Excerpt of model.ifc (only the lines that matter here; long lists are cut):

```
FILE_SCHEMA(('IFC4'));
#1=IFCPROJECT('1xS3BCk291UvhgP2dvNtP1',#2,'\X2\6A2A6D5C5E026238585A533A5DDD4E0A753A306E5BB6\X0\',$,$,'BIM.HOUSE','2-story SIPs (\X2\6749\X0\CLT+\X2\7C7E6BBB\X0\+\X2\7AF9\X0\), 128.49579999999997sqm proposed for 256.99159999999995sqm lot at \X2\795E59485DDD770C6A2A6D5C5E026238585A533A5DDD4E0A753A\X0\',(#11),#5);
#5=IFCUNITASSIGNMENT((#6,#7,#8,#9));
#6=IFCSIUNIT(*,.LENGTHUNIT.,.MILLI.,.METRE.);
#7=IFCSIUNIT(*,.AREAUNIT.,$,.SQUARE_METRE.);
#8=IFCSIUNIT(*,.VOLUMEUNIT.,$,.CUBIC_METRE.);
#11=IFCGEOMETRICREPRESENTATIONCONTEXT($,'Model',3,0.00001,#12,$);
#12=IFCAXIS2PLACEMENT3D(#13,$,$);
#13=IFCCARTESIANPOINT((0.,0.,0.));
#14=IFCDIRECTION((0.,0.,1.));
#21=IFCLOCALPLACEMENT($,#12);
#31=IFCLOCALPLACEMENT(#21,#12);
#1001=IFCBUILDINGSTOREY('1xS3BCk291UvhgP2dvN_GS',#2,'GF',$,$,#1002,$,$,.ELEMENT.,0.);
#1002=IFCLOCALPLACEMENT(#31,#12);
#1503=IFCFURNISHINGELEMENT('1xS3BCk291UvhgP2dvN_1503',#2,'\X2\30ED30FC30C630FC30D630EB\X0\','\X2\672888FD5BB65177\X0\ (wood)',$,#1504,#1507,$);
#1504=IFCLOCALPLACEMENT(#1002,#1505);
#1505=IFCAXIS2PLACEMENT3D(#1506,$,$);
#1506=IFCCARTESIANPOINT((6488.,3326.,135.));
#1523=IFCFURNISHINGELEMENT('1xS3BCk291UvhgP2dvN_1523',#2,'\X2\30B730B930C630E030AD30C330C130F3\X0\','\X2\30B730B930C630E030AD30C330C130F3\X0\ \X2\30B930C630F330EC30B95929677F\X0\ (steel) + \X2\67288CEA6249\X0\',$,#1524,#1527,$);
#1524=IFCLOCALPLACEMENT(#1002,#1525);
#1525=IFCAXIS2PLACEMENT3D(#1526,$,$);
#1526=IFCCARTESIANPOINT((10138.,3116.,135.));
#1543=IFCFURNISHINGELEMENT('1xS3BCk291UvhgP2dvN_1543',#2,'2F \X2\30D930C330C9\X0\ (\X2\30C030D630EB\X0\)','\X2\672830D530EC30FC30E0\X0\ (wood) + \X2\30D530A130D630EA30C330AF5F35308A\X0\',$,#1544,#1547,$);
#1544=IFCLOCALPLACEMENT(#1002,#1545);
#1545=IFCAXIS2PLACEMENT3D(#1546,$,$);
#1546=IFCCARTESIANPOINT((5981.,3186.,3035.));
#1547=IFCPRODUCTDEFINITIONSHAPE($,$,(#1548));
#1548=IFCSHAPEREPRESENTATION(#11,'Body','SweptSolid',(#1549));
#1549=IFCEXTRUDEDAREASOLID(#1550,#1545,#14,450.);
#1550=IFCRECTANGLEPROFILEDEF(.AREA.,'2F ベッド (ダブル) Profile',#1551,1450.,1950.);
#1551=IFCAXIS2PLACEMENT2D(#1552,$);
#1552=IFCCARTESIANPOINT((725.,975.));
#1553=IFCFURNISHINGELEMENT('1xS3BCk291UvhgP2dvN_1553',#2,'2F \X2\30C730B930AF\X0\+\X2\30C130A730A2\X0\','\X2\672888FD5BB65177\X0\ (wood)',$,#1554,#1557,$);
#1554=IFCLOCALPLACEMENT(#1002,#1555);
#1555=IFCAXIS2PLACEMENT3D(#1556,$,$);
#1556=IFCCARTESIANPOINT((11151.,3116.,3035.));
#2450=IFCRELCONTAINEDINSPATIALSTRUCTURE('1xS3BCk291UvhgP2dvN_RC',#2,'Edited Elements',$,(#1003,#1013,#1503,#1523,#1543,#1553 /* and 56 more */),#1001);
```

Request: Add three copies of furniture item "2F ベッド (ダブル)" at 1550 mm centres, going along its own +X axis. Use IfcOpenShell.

```python
import ifcopenshell
import ifcopenshell.api.geometry
import ifcopenshell.api.root
import ifcopenshell.util.element
import ifcopenshell.util.placement
import ifcopenshell.util.unit

model = ifcopenshell.open("model.ifc")
unit_scale = ifcopenshell.util.unit.calculate_unit_scale(model)


def reuse_history(source, copy):
    """copy_class also copies each property set's owner history, people and application; keep the originals."""
    for rel in copy.IsDefinedBy:
        if rel.is_a("IfcRelDefinesByProperties") and (history := rel.RelatingPropertyDefinition.OwnerHistory):
            rel.RelatingPropertyDefinition.OwnerHistory = source.OwnerHistory
            ifcopenshell.util.element.remove_deep2(model, history)


source = model.by_guid("1xS3BCk291UvhgP2dvN_1543")
base = ifcopenshell.util.placement.get_local_placement(source.ObjectPlacement)
step = base[:3, 0] * 1.55 / unit_scale

for i in range(1, 4):
    copy = ifcopenshell.api.root.copy_class(model, product=source)
    copy.Representation = ifcopenshell.util.element.copy_deep(
        model, source.Representation, exclude=["IfcGeometricRepresentationContext", "IfcRepresentationMap"]
    )
    reuse_history(source, copy)
    matrix = base.copy()
    matrix[:3, 3] += i * step
    print("added at", matrix[:3, 3].round(3) + 0.0)
    ifcopenshell.api.geometry.edit_object_placement(model, product=copy, matrix=matrix, is_si=False)

model.write("model_updated.ifc")
```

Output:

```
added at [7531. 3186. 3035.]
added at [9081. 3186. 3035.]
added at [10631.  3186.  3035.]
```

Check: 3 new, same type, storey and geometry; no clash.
